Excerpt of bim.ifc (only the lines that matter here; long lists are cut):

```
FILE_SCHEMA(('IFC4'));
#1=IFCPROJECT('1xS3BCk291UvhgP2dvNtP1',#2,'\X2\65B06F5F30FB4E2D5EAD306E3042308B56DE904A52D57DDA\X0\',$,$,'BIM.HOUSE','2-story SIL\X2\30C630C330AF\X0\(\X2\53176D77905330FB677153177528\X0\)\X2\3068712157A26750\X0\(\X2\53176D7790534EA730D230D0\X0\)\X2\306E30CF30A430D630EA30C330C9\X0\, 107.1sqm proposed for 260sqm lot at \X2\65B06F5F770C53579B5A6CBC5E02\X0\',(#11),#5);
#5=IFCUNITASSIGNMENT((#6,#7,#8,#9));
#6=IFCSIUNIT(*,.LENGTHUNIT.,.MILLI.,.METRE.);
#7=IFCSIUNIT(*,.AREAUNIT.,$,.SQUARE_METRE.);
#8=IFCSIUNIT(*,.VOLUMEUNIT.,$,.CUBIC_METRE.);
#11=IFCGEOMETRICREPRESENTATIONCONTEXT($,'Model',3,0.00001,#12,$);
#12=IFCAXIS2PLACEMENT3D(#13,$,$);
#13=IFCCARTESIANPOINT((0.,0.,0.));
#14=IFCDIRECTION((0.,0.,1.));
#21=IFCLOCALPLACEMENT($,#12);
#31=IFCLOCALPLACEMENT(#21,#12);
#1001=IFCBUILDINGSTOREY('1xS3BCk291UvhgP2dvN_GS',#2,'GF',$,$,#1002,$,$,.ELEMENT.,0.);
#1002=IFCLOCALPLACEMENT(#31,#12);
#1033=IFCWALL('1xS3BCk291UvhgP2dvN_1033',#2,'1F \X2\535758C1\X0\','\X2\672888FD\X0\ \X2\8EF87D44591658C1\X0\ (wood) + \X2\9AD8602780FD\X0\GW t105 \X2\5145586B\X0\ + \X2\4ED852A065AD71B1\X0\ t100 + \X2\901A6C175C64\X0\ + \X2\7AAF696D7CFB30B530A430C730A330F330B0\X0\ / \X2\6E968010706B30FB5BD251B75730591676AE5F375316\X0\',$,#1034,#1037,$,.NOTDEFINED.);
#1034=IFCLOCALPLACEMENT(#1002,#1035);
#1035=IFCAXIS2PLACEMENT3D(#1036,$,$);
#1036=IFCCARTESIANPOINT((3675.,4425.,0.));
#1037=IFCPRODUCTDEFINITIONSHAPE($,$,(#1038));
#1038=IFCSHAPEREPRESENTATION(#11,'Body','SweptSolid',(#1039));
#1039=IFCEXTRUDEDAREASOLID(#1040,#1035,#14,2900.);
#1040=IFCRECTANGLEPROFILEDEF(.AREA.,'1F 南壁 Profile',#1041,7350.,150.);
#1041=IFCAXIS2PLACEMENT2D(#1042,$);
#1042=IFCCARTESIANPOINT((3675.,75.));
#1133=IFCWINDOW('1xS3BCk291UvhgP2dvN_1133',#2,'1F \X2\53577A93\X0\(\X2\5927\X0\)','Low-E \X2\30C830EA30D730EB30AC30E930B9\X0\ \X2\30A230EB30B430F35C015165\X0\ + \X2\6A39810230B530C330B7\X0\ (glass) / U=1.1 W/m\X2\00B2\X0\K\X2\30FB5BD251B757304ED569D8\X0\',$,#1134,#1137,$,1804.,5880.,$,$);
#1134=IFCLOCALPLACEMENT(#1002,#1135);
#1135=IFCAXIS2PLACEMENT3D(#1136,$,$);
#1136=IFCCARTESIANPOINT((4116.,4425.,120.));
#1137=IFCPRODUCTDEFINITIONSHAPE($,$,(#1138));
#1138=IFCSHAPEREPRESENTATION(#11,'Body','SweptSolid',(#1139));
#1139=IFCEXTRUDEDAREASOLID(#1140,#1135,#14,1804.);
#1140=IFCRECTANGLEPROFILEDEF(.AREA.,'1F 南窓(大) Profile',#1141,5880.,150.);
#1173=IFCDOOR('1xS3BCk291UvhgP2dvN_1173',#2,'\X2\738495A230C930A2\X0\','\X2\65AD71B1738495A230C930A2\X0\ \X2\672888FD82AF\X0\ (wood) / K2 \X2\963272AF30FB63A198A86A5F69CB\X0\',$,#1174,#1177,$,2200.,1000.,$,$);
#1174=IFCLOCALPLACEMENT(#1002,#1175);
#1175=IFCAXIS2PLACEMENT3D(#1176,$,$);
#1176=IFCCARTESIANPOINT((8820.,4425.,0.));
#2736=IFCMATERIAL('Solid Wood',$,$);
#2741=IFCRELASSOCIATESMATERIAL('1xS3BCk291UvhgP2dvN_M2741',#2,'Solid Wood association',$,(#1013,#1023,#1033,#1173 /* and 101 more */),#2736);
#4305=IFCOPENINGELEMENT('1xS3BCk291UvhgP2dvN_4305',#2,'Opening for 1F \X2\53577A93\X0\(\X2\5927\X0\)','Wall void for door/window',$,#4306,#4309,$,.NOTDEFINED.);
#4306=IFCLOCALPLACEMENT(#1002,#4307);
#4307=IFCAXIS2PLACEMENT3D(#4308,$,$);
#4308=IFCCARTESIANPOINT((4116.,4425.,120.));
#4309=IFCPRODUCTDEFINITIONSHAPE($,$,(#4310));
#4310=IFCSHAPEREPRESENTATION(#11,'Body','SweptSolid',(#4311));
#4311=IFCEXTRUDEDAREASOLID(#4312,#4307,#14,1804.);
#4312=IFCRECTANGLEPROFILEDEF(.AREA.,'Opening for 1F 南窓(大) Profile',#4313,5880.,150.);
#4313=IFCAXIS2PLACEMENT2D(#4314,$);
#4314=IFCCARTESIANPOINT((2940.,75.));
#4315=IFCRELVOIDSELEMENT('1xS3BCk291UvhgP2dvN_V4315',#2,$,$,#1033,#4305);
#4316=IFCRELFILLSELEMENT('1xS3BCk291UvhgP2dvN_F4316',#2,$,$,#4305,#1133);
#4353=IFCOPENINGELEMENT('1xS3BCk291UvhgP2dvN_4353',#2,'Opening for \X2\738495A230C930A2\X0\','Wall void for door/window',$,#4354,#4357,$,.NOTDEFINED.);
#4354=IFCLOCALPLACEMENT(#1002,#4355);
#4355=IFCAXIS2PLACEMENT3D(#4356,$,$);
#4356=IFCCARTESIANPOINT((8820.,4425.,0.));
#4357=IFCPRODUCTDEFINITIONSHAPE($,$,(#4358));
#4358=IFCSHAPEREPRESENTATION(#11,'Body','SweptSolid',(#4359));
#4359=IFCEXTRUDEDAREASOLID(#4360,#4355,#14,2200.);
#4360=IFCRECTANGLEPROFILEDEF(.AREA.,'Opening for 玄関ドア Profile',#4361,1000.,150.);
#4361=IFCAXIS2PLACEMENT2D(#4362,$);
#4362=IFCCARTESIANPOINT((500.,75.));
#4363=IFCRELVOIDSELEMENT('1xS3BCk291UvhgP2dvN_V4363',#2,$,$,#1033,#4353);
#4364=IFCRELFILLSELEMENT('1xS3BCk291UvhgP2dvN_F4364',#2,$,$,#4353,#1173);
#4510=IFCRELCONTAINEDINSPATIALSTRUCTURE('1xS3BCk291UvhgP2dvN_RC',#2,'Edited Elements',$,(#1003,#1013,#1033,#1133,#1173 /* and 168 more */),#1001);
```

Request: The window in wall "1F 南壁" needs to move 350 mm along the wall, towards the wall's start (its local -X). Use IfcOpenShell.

```python
import ifcopenshell
import ifcopenshell.api.geometry
import ifcopenshell.util.placement
import ifcopenshell.util.unit

model = ifcopenshell.open("bim.ifc")
unit_scale = ifcopenshell.util.unit.calculate_unit_scale(model)

window = model.by_guid("1xS3BCk291UvhgP2dvN_1133")
opening = window.FillsVoids[0].RelatingOpeningElement
wall = opening.VoidsElements[0].RelatingBuildingElement

wall_matrix = ifcopenshell.util.placement.get_local_placement(wall.ObjectPlacement)
shift = wall_matrix[:3, 0] * -0.35 / unit_scale
before = ifcopenshell.util.placement.get_local_placement(window.ObjectPlacement)[:3, 3].copy()

# The window is not placed relative to its opening, so move both.
for product in (opening, window):
    matrix = ifcopenshell.util.placement.get_local_placement(product.ObjectPlacement)
    matrix[:3, 3] += shift
    ifcopenshell.api.geometry.edit_object_placement(model, product=product, matrix=matrix, is_si=False)

after = ifcopenshell.util.placement.get_local_placement(window.ObjectPlacement)[:3, 3]
print("window moved by", (after - before).round(3) + 0.0)

model.write("bim_v2.ifc")
```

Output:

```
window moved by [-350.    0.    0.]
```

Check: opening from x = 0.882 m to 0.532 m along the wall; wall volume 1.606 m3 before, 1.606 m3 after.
